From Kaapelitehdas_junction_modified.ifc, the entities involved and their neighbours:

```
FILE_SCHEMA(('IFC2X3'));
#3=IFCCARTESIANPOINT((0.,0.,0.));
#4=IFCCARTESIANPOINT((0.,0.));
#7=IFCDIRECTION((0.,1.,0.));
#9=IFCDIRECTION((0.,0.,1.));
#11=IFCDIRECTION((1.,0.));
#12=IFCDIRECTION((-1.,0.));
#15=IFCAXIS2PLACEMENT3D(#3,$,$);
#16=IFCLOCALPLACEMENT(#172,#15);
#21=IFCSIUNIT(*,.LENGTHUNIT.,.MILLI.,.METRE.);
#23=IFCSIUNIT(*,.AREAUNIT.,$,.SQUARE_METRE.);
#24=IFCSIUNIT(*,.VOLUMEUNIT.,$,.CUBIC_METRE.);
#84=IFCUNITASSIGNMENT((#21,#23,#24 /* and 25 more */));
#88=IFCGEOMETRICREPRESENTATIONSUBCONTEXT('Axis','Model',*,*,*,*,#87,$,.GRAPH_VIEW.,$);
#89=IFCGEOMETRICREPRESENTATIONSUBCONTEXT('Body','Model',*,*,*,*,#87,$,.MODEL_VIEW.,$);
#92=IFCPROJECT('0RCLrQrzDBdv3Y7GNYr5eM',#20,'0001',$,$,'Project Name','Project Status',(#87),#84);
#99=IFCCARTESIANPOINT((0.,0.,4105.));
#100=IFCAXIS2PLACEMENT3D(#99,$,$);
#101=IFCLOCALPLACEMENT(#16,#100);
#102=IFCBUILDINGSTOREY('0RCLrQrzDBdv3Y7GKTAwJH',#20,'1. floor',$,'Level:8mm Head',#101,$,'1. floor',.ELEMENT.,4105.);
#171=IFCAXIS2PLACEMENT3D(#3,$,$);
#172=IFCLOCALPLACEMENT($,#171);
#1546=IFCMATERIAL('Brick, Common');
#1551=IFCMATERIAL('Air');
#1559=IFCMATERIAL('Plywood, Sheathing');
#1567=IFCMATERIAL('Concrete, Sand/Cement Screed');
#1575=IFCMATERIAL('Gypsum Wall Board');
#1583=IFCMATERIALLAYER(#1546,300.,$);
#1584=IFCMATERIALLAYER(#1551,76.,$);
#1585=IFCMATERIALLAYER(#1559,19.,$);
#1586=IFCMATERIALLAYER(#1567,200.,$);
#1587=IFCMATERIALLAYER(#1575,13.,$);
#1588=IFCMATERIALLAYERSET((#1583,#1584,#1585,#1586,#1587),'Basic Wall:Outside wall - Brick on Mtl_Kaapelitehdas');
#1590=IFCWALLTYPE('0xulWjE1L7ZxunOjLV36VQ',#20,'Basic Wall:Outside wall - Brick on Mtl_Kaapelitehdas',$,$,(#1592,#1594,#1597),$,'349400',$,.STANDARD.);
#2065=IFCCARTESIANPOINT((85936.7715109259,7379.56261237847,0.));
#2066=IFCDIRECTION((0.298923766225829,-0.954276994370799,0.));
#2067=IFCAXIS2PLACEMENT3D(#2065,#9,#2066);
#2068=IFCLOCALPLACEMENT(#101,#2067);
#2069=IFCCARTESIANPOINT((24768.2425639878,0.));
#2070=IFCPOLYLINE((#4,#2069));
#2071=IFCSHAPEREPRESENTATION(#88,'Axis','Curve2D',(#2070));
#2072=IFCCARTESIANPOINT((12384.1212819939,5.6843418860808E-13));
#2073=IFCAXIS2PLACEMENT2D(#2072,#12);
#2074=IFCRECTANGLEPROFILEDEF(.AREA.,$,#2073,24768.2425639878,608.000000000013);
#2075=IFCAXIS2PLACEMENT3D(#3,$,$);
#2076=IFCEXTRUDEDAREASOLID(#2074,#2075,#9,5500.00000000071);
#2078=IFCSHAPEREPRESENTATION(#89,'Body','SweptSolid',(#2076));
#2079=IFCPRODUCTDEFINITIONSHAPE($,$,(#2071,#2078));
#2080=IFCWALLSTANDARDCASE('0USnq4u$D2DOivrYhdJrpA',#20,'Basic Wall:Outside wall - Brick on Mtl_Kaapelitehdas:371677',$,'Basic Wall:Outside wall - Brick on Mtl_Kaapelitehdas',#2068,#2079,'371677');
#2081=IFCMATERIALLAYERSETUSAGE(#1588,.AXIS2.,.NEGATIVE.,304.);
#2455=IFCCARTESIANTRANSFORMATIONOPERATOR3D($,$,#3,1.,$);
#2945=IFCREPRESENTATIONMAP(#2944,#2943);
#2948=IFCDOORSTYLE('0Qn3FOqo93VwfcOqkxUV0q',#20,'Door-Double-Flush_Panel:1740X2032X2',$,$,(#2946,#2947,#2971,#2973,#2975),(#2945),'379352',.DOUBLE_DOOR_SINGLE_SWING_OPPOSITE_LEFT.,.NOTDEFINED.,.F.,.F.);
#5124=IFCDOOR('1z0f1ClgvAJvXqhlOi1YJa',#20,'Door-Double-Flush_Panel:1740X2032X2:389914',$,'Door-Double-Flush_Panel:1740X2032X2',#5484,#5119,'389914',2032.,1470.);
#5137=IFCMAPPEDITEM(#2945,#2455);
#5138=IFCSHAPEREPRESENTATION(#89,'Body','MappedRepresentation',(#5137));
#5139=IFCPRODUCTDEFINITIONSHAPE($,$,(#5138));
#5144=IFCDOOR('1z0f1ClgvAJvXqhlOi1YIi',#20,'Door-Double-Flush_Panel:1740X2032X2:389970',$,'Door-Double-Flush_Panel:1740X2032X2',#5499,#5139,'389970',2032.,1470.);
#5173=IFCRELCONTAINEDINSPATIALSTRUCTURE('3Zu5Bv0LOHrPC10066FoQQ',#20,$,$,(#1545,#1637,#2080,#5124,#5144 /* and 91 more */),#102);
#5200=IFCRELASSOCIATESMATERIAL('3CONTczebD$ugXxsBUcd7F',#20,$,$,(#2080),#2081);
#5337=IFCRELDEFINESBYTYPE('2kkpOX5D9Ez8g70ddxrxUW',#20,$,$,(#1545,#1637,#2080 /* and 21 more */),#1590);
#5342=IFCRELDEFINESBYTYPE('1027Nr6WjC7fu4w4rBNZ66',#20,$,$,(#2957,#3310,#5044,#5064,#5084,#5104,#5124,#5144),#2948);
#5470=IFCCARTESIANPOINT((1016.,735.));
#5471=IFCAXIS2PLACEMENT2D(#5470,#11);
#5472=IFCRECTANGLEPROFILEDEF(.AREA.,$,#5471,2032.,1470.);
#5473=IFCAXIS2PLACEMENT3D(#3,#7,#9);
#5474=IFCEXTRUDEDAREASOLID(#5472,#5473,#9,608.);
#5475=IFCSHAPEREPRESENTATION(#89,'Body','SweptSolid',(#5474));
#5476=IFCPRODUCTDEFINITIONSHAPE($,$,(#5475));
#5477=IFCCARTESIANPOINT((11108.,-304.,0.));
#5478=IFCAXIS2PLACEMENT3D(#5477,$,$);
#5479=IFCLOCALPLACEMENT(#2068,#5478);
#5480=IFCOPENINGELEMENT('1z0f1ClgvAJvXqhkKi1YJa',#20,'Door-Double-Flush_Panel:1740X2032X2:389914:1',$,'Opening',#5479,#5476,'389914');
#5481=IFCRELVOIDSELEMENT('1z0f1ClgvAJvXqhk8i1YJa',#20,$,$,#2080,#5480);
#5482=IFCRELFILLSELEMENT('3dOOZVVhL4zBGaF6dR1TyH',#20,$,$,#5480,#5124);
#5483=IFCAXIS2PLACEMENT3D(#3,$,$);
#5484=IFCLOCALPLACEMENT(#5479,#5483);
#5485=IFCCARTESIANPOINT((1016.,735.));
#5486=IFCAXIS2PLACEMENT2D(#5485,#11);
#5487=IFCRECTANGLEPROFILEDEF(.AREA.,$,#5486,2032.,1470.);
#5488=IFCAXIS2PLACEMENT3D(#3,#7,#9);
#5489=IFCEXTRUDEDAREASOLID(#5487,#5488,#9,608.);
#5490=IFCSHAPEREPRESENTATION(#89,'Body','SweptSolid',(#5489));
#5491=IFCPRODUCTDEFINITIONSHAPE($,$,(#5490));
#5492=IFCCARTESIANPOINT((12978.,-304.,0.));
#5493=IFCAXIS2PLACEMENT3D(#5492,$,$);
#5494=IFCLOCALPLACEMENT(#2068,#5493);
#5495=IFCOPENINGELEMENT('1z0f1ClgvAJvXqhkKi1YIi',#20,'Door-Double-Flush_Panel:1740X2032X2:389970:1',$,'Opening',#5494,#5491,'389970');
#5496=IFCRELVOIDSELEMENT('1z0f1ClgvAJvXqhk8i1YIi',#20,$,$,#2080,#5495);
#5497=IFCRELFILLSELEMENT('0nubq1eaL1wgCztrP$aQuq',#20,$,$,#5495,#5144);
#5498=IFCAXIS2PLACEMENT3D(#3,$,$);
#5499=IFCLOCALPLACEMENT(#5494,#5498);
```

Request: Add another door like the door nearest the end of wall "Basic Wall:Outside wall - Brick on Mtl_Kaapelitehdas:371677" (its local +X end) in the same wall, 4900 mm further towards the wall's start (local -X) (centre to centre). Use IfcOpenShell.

```python
import ifcopenshell
import ifcopenshell.api.feature
import ifcopenshell.api.geometry
import ifcopenshell.api.root
import ifcopenshell.geom
import ifcopenshell.util.element
import ifcopenshell.util.placement
import ifcopenshell.util.shape
import ifcopenshell.util.unit

model = ifcopenshell.open("Kaapelitehdas_junction_modified.ifc")
unit_scale = ifcopenshell.util.unit.calculate_unit_scale(model)
settings = ifcopenshell.geom.settings()


def volume(element):
    """Net volume in cubic metres, openings subtracted."""
    shape = ifcopenshell.geom.create_shape(settings, element)
    return ifcopenshell.util.shape.get_volume(shape.geometry)


def reuse_history(source, copy):
    """copy_class also copies each property set's owner history, people and application; keep the originals."""
    for rel in copy.IsDefinedBy:
        if rel.is_a("IfcRelDefinesByProperties") and (history := rel.RelatingPropertyDefinition.OwnerHistory):
            rel.RelatingPropertyDefinition.OwnerHistory = source.OwnerHistory
            ifcopenshell.util.element.remove_deep2(model, history)


door = model.by_guid("1z0f1ClgvAJvXqhlOi1YIi")
opening = door.FillsVoids[0].RelatingOpeningElement
wall = opening.VoidsElements[0].RelatingBuildingElement
before = volume(wall)
shift = ifcopenshell.util.placement.get_local_placement(wall.ObjectPlacement)[:3, 0] * -4.9 / unit_scale

# copy_class copies the void relationship, type, container and properties, but no geometry.
new_opening = ifcopenshell.api.root.copy_class(model, product=opening)
new_opening.Representation = ifcopenshell.util.element.copy_deep(
    model, opening.Representation, exclude=["IfcGeometricRepresentationContext", "IfcRepresentationMap"]
)
new_opening.Name = "Door-Double-Flush_Panel:1740X2032X2"
new_opening.Tag = None
new_door = ifcopenshell.api.root.copy_class(model, product=door)
new_door.Representation = ifcopenshell.util.element.copy_deep(
    model, door.Representation, exclude=["IfcGeometricRepresentationContext", "IfcRepresentationMap"]
)
new_door.Name = "Door-Double-Flush_Panel:1740X2032X2"
new_door.Tag = None
reuse_history(door, new_door)
fills = ifcopenshell.api.feature.add_filling(model, opening=new_opening, element=new_door)
fills.OwnerHistory = new_door.OwnerHistory  # required in IFC2X3

for old, new in ((opening, new_opening), (door, new_door)):
    matrix = ifcopenshell.util.placement.get_local_placement(old.ObjectPlacement)
    matrix[:3, 3] += shift
    ifcopenshell.api.geometry.edit_object_placement(model, product=new, matrix=matrix, is_si=False)

after = volume(wall)

print(f"wall volume {before:.3f} -> {after:.3f} m3")

model.write("Kaapelitehdas_junction_modified_edited.ifc")
```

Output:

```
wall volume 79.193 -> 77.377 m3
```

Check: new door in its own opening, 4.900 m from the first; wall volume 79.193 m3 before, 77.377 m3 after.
